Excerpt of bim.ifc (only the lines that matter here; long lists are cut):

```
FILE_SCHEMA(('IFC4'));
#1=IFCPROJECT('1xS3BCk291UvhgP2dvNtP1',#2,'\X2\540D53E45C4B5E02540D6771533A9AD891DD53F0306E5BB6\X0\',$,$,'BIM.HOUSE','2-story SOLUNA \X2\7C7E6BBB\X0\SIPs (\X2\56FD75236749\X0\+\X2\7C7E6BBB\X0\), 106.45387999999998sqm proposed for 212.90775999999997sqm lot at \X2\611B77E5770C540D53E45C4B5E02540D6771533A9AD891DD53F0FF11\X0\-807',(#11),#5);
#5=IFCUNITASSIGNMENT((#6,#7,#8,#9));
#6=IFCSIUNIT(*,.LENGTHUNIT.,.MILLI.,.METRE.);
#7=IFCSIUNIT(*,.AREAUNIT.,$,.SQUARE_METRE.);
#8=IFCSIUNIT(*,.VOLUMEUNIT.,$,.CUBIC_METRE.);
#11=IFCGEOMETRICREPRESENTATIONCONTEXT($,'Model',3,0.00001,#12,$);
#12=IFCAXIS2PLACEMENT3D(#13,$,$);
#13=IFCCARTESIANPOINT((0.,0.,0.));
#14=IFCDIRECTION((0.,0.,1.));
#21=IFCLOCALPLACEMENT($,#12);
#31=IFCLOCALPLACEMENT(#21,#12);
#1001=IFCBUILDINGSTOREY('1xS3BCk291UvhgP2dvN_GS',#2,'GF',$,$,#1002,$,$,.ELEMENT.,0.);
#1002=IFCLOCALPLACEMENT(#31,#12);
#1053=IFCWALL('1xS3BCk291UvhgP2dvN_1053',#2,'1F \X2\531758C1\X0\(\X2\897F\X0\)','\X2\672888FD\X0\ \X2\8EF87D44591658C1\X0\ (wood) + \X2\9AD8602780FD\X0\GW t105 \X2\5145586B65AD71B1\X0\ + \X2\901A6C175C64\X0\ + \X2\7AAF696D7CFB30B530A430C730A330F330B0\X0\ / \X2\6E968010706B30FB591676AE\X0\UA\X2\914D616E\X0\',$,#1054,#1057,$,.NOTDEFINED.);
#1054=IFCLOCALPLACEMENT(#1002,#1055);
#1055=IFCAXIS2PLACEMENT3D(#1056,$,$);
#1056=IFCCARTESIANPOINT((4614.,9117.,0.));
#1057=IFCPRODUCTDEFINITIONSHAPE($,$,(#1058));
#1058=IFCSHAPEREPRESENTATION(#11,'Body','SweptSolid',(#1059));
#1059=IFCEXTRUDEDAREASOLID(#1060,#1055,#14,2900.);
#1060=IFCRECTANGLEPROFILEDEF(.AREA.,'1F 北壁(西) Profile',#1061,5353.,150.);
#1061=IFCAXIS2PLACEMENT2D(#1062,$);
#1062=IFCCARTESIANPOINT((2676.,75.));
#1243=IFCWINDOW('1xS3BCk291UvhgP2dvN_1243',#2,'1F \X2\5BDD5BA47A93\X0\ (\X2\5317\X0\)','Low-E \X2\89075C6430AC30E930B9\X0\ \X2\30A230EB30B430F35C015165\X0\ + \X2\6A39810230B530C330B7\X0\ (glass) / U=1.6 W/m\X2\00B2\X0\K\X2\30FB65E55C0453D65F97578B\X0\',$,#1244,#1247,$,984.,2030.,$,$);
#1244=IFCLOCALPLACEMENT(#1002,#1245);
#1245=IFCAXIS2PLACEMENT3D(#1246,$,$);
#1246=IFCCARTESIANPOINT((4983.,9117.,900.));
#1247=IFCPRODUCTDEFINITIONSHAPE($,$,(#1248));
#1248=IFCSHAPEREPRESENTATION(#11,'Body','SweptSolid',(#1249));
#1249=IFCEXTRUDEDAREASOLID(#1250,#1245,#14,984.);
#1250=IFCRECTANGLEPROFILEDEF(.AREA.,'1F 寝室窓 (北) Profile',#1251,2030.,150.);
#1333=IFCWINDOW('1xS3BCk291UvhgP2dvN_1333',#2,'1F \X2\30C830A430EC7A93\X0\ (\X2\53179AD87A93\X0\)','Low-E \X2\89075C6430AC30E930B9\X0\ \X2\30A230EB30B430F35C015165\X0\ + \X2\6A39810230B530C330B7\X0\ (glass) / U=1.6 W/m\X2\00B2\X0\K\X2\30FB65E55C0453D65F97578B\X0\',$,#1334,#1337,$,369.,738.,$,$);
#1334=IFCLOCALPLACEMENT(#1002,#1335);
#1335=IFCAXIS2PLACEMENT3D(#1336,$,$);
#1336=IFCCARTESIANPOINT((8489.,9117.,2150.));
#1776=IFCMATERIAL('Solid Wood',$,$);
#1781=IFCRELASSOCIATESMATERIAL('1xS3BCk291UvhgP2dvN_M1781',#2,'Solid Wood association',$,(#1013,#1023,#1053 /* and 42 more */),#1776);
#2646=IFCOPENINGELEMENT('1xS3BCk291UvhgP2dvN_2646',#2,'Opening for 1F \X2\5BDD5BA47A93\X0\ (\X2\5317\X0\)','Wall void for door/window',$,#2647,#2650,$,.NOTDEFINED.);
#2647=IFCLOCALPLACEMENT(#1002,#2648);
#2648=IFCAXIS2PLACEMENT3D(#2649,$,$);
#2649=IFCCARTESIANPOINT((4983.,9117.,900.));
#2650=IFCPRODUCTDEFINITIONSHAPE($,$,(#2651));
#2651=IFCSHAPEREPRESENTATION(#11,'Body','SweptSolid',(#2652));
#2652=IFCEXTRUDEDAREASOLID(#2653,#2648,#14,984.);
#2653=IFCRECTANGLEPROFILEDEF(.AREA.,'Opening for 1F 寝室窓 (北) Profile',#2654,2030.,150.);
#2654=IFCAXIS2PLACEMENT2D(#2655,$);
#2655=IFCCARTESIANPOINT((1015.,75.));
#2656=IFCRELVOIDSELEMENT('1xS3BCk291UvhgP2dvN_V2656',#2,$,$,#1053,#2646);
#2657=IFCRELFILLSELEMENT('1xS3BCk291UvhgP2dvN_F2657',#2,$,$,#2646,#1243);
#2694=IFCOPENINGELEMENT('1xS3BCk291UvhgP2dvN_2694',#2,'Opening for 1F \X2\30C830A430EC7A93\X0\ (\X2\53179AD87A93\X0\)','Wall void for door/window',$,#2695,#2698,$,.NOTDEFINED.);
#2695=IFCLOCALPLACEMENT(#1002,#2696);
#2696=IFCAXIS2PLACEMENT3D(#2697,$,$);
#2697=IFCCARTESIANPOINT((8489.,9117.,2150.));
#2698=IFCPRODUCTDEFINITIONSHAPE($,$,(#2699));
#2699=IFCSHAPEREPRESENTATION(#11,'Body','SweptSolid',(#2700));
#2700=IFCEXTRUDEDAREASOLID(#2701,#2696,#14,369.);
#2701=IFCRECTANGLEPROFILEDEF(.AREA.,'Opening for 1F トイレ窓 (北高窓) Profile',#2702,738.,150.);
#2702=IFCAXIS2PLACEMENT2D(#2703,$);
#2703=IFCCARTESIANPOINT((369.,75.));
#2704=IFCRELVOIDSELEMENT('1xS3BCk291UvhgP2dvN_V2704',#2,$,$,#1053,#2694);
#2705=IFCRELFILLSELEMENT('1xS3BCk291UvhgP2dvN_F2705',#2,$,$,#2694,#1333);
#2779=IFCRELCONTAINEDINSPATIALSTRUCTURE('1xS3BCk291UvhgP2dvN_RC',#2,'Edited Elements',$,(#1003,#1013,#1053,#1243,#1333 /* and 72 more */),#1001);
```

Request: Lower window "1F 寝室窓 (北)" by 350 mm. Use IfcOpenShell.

```python
import numpy as np
import ifcopenshell
import ifcopenshell.api.geometry
import ifcopenshell.util.placement
import ifcopenshell.util.unit

model = ifcopenshell.open("bim.ifc")
unit_scale = ifcopenshell.util.unit.calculate_unit_scale(model)

window = model.by_guid("1xS3BCk291UvhgP2dvN_1243")
opening = window.FillsVoids[0].RelatingOpeningElement
dz = -350.0

shift = np.array([0.0, 0.0, dz])
# The window is not placed relative to its opening, so move both.
for product in (opening, window):
    matrix = ifcopenshell.util.placement.get_local_placement(product.ObjectPlacement)
    matrix[:3, 3] += shift
    ifcopenshell.api.geometry.edit_object_placement(model, product=product, matrix=matrix, is_si=False)

print(f"moved by {dz * unit_scale:+.3f} m")

model.write("bim_edited.ifc")
```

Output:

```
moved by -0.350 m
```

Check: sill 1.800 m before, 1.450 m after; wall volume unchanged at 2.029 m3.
